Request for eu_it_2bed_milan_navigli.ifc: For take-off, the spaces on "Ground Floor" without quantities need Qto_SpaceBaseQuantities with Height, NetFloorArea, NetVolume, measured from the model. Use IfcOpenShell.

First a look at what the model holds.

```python
import ifcopenshell
import ifcopenshell.util.element
import ifcopenshell.util.unit

model = ifcopenshell.open("eu_it_2bed_milan_navigli.ifc")
print(model.schema)
for unit_type in ("LENGTHUNIT", "AREAUNIT", "VOLUMEUNIT"):
    print(unit_type, ifcopenshell.util.unit.calculate_unit_scale(model, unit_type))
storey = next(s for s in model.by_type("IfcBuildingStorey") if s.Name == "Ground Floor")
spaces = [e for e in ifcopenshell.util.element.get_decomposition(storey) if e.is_a("IfcSpace")]
for e in sorted(spaces, key=lambda e: e.id()):
    print(e.id(), e.is_a(), e.Name, list(ifcopenshell.util.element.get_psets(e, qtos_only=True)), sep=" | ")
```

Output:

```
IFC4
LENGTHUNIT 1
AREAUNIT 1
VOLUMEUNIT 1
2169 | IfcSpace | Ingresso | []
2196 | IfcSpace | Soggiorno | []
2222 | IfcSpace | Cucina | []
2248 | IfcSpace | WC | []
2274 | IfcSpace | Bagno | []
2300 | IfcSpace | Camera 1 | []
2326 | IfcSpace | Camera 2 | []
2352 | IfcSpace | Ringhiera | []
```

```python
import ifcopenshell
import ifcopenshell.api.pset
import ifcopenshell.geom
import ifcopenshell.util.element
import ifcopenshell.util.shape
import ifcopenshell.util.unit

model = ifcopenshell.open("eu_it_2bed_milan_navigli.ifc")
unit_scale = ifcopenshell.util.unit.calculate_unit_scale(model)
area_scale = ifcopenshell.util.unit.calculate_unit_scale(model, "AREAUNIT")
volume_scale = ifcopenshell.util.unit.calculate_unit_scale(model, "VOLUMEUNIT")
settings = ifcopenshell.geom.settings()

storey = next(s for s in model.by_type("IfcBuildingStorey") if s.Name == "Ground Floor")
spaces = [e for e in ifcopenshell.util.element.get_decomposition(storey) if e.is_a("IfcSpace")]

for e in sorted(spaces, key=lambda e: e.id()):
    if ifcopenshell.util.element.get_psets(e, qtos_only=True, should_inherit=False):
        continue
    # Geometry comes back in metres, in the element's own axes.
    shape = ifcopenshell.geom.create_shape(settings, e)
    values = {
        "Height": ifcopenshell.util.shape.get_z(shape.geometry) / unit_scale,
        "NetFloorArea": ifcopenshell.util.shape.get_footprint_area(shape.geometry) / area_scale,
        "NetVolume": ifcopenshell.util.shape.get_volume(shape.geometry) / volume_scale,
    }
    qto = ifcopenshell.api.pset.add_qto(model, product=e, name="Qto_SpaceBaseQuantities")
    ifcopenshell.api.pset.edit_qto(model, qto=qto, properties=values)
    print(e.id(), {k: round(v, 3) for k, v in values.items()})

model.write("eu_it_2bed_milan_navigli_edited.ifc")
```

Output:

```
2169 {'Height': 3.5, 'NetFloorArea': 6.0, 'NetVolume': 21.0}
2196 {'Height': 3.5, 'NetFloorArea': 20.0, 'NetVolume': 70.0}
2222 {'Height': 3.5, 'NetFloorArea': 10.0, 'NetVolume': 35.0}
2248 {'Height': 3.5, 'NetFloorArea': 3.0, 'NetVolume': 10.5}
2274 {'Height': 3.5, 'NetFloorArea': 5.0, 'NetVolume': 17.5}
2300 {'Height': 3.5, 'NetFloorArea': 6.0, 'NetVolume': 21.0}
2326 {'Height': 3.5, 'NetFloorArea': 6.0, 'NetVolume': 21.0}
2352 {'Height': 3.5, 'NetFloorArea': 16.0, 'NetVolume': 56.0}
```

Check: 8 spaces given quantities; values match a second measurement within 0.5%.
